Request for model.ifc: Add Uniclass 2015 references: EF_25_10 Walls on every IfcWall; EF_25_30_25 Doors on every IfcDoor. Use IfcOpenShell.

First a look at what the model holds.

```python
import ifcopenshell

model = ifcopenshell.open("model.ifc")
print(model.schema)
print("classifications:", [c.Name for c in model.by_type("IfcClassification")])
for ifc_class in ("IfcDoor", "IfcRoof", "IfcStair", "IfcWall", "IfcWindow"):
    print(ifc_class, len(model.by_type(ifc_class)))
```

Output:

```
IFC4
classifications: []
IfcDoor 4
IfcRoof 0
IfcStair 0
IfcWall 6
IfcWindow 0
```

```python
import ifcopenshell
import ifcopenshell.api.classification

model = ifcopenshell.open("model.ifc")

system = ifcopenshell.api.classification.add_classification(model, classification="Uniclass 2015")

codes = {
    "IfcWall": ("EF_25_10", "Walls"),
    "IfcDoor": ("EF_25_30_25", "Doors"),
}
for ifc_class, (code, name) in codes.items():
    products = model.by_type(ifc_class)
    ifcopenshell.api.classification.add_reference(
        model, products=products, classification=system, identification=code, name=name
    )
    print(code, len(products))

model.write("model_rev.ifc")
```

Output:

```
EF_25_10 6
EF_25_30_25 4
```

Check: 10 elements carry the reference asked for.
